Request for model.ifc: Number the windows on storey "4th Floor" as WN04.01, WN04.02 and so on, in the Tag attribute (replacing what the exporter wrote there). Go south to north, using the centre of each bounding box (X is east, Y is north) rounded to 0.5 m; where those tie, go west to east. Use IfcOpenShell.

First a look at what the model holds.

```python
import ifcopenshell
import ifcopenshell.util.element
import ifcopenshell.util.placement

model = ifcopenshell.open("model.ifc")
print(model.schema)
storey = next(s for s in model.by_type("IfcBuildingStorey") if s.Name == "4th Floor")
windows = [e for e in ifcopenshell.util.element.get_decomposition(storey) if e.is_a("IfcWindow")]
for e in sorted(windows, key=lambda e: e.id()):
    origin = ifcopenshell.util.placement.get_local_placement(e.ObjectPlacement)[:3, 3]
    print(e.id(), e.Tag, e.Name, origin.round(2) + 0.0, sep=" | ")
```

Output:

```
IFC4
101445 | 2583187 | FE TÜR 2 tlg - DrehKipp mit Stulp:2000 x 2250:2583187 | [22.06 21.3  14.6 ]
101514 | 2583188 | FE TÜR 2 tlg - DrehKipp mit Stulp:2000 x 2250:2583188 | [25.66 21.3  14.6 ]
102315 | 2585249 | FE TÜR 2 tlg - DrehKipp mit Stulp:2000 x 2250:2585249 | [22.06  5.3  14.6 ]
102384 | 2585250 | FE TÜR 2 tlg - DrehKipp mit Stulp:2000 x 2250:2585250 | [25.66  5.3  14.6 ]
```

```python
import ifcopenshell
import ifcopenshell.geom
import ifcopenshell.util.element
import ifcopenshell.util.shape

model = ifcopenshell.open("model.ifc")
settings = ifcopenshell.geom.settings()
settings.set("use-world-coords", True)


def centre(element):
    shape = ifcopenshell.geom.create_shape(settings, element)
    return ifcopenshell.util.shape.get_bbox_centroid(shape.geometry)


storey = next(s for s in model.by_type("IfcBuildingStorey") if s.Name == "4th Floor")
windows = [e for e in ifcopenshell.util.element.get_decomposition(storey) if e.is_a("IfcWindow")]

# Insertion points can sit at a corner or the storey origin, so sort by the geometry (in metres).
centres = {e: centre(e) for e in windows}
windows.sort(key=lambda e: (round(centres[e][1] / 0.5), centres[e][0]))

for i, e in enumerate(windows, start=1):
    number = f"WN04.{i:02d}"
    e.Tag = number
    print(e.id(), number)

model.write("model_v2.ifc")
```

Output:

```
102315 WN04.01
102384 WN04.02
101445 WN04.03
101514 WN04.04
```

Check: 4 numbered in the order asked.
